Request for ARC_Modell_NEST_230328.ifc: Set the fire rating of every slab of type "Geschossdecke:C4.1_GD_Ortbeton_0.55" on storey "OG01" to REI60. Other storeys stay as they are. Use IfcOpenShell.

First a look at what the model holds.

```python
import ifcopenshell
import ifcopenshell.util.element

model = ifcopenshell.open("ARC_Modell_NEST_230328.ifc")
print(model.schema)
storey = next(s for s in model.by_type("IfcBuildingStorey") if s.Name == "OG01")
slabs = [e for e in ifcopenshell.util.element.get_decomposition(storey) if e.is_a("IfcSlab")]
seen = {}
for e in slabs:
    element_type = ifcopenshell.util.element.get_type(e)
    key = (element_type.Name if element_type != e and element_type else None, ifcopenshell.util.element.get_pset(e, "Pset_SlabCommon", "FireRating"))
    seen[key] = seen.get(key, 0) + 1
for (name, value), count in sorted(seen.items(), key=str):
    print(count, "x", name, "|", value)
```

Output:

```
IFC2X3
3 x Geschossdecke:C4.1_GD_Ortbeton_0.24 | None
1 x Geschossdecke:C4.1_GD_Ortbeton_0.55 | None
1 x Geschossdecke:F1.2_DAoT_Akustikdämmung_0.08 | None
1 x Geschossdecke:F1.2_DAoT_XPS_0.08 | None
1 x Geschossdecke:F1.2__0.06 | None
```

```python
import ifcopenshell
import ifcopenshell.api.pset
import ifcopenshell.util.element

model = ifcopenshell.open("ARC_Modell_NEST_230328.ifc")

storey = next(s for s in model.by_type("IfcBuildingStorey") if s.Name == "OG01")
slabs = [e for e in ifcopenshell.util.element.get_decomposition(storey) if e.is_a("IfcSlab")]

count = 0
for e in slabs:
    element_type = ifcopenshell.util.element.get_type(e)
    if element_type in (None, e) or element_type.Name != "Geschossdecke:C4.1_GD_Ortbeton_0.55":
        continue
    # add_pset returns the element's existing set when there is one.
    pset = ifcopenshell.api.pset.add_pset(model, product=e, name="Pset_SlabCommon")
    ifcopenshell.api.pset.edit_pset(model, pset=pset, properties={"FireRating": "REI60"})
    count += 1

print(count, "slabs updated")

model.write("ARC_Modell_NEST_230328_rev.ifc")
```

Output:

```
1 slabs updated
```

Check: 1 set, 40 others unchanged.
